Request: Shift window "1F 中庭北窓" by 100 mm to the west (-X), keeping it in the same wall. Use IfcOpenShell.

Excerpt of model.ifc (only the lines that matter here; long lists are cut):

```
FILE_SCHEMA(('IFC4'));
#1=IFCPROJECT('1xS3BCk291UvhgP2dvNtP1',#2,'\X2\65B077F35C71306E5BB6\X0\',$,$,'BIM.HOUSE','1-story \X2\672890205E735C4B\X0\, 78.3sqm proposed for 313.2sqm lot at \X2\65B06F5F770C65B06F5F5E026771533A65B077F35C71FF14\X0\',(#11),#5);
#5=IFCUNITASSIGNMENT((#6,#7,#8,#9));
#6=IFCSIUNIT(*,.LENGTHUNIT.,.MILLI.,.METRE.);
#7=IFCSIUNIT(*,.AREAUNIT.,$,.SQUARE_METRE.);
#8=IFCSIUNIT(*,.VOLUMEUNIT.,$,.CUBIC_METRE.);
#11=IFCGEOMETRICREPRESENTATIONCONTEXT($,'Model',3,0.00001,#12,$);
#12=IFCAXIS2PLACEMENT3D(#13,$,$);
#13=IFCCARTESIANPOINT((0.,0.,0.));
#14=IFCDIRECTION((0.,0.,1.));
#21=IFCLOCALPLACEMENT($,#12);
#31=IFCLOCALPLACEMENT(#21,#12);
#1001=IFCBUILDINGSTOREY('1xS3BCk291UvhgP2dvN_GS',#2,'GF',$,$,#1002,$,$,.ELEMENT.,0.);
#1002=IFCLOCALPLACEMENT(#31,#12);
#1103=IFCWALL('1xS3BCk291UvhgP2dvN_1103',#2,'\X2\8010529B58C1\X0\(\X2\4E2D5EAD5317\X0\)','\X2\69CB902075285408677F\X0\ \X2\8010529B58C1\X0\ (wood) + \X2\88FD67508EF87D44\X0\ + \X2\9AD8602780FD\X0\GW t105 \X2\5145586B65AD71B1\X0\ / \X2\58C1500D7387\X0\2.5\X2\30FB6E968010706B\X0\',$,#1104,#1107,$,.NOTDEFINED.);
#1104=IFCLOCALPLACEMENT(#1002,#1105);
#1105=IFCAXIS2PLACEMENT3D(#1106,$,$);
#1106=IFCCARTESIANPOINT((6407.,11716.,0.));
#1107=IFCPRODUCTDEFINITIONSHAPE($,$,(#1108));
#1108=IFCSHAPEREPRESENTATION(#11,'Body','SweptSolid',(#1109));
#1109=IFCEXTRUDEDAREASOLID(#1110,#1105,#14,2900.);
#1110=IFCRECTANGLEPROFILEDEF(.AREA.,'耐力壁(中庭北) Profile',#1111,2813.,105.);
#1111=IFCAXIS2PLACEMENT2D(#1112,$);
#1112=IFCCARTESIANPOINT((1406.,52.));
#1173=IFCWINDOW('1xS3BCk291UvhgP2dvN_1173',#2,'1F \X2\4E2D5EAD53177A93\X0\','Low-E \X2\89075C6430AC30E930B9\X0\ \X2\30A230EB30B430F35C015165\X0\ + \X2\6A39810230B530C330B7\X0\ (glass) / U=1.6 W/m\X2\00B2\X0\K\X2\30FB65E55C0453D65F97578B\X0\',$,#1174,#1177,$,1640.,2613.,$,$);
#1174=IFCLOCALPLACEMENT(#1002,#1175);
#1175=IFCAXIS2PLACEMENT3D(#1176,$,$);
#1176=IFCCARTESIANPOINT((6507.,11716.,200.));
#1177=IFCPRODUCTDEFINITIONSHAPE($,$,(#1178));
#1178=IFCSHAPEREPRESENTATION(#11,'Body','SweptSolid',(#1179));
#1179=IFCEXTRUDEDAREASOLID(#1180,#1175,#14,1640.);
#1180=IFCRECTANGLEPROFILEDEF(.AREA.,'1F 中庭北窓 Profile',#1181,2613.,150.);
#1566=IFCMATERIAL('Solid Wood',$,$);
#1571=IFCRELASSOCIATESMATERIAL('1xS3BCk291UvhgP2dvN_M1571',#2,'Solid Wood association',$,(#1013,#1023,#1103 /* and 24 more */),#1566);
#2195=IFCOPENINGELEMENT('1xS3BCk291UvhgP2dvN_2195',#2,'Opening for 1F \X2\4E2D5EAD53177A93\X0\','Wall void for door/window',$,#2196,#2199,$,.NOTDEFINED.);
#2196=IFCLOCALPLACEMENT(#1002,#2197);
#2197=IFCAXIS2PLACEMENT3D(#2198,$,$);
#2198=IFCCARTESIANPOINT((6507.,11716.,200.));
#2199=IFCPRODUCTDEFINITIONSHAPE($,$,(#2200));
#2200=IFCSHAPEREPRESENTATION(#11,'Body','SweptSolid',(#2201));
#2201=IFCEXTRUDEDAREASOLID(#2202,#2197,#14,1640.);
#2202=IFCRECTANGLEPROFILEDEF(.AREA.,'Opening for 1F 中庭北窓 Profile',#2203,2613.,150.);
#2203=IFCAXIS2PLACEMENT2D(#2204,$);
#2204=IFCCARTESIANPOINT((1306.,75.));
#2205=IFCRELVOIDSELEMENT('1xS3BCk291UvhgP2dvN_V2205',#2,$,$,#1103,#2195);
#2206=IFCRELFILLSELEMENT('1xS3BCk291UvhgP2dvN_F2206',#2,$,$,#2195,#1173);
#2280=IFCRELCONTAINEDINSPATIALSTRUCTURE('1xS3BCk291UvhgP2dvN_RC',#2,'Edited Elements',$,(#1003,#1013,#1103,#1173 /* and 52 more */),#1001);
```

```python
import ifcopenshell
import ifcopenshell.api.geometry
import ifcopenshell.util.placement

model = ifcopenshell.open("model.ifc")

window = model.by_guid("1xS3BCk291UvhgP2dvN_1173")
opening = window.FillsVoids[0].RelatingOpeningElement
wall = opening.VoidsElements[0].RelatingBuildingElement

wall_matrix = ifcopenshell.util.placement.get_local_placement(wall.ObjectPlacement)
shift = wall_matrix[:3, 0] * -100.0
before = ifcopenshell.util.placement.get_local_placement(window.ObjectPlacement)[:3, 3].copy()

# The window is not placed relative to its opening, so move both.
for product in (opening, window):
    matrix = ifcopenshell.util.placement.get_local_placement(product.ObjectPlacement)
    matrix[:3, 3] += shift
    ifcopenshell.api.geometry.edit_object_placement(model, product=product, matrix=matrix, is_si=False)

after = ifcopenshell.util.placement.get_local_placement(window.ObjectPlacement)[:3, 3]
print("window moved by", (after - before).round(3) + 0.0)

model.write("model_updated.ifc")
```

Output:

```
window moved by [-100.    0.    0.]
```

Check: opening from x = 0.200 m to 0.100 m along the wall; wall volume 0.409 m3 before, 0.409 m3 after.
